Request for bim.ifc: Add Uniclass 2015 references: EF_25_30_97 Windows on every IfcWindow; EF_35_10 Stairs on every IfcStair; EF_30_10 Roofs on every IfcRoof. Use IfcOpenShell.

First a look at what the model holds.

```python
import ifcopenshell

model = ifcopenshell.open("bim.ifc")
print(model.schema)
print("classifications:", [c.Name for c in model.by_type("IfcClassification")])
for ifc_class in ("IfcDoor", "IfcRoof", "IfcStair", "IfcWall", "IfcWindow"):
    print(ifc_class, len(model.by_type(ifc_class)))
```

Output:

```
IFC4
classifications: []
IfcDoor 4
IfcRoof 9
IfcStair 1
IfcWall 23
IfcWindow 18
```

```python
import ifcopenshell
import ifcopenshell.api.classification

model = ifcopenshell.open("bim.ifc")

system = ifcopenshell.api.classification.add_classification(model, classification="Uniclass 2015")

codes = {
    "IfcWindow": ("EF_25_30_97", "Windows"),
    "IfcStair": ("EF_35_10", "Stairs"),
    "IfcRoof": ("EF_30_10", "Roofs"),
}
for ifc_class, (code, name) in codes.items():
    products = model.by_type(ifc_class)
    ifcopenshell.api.classification.add_reference(
        model, products=products, classification=system, identification=code, name=name
    )
    print(code, len(products))

model.write("bim-out.ifc")
```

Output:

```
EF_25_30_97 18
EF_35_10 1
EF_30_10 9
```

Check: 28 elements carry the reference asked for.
